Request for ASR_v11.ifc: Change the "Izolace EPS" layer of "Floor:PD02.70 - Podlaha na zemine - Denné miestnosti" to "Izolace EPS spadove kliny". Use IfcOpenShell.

First a look at what the model holds.

```python
import ifcopenshell
import ifcopenshell.util.element

model = ifcopenshell.open("ASR_v11.ifc")
print(model.schema)
for layer_set in model.by_type("IfcMaterialLayerSet"):
    if layer_set.LayerSetName == "Floor:PD02.70 - Podlaha na zemine - Denné miestnosti":
        for layer in layer_set.MaterialLayers:
            print(layer.id(), layer.Material and layer.Material.Name, layer.LayerThickness, sep=" | ")
        print(len(ifcopenshell.util.element.get_elements_by_material(model, layer_set)), "elements and types use it")
print(sorted(m.Name for m in model.by_type("IfcMaterial") if m.Name)[:60])
```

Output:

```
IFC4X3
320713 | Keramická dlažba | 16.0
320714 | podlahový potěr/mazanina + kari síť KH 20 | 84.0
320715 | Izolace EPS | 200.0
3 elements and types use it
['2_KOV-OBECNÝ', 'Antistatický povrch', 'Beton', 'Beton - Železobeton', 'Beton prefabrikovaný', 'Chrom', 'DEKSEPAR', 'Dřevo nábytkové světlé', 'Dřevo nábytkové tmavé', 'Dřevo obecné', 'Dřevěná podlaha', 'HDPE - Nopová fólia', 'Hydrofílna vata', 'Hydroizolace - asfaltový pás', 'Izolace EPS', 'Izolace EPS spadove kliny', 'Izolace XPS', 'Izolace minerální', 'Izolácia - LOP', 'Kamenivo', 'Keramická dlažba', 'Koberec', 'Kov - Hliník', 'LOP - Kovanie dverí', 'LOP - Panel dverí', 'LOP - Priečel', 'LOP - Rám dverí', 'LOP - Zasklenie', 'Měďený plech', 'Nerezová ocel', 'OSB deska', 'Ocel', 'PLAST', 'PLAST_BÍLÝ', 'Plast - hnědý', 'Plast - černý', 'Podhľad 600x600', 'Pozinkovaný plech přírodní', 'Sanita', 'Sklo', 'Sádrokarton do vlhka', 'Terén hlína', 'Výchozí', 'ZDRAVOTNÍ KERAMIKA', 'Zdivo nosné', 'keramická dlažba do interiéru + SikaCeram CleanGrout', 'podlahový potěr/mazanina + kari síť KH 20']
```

```python
import ifcopenshell
import ifcopenshell.api.material

model = ifcopenshell.open("ASR_v11.ifc")

layer_set = next(s for s in model.by_type("IfcMaterialLayerSet") if s.LayerSetName == "Floor:PD02.70 - Podlaha na zemine - Denné miestnosti")
layer = next(l for l in layer_set.MaterialLayers if l.Material and l.Material.Name == "Izolace EPS")
material = next(m for m in model.by_type("IfcMaterial") if m.Name == "Izolace EPS spadove kliny")

# Point this one layer at the other material; renaming the old one would change it everywhere.
ifcopenshell.api.material.edit_layer(model, layer=layer, attributes={"Name": material.Name}, material=material)

print([l.Material.Name if l.Material else None for l in layer_set.MaterialLayers])

model.write("ASR_v11_updated.ifc")
```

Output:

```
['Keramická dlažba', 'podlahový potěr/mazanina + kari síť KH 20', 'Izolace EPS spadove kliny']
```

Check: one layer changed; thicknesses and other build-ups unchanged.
